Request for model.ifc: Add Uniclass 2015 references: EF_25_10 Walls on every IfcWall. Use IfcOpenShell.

First a look at what the model holds.

```python
import ifcopenshell

model = ifcopenshell.open("model.ifc")
print(model.schema)
print("classifications:", [c.Name for c in model.by_type("IfcClassification")])
for ifc_class in ("IfcDoor", "IfcRoof", "IfcStair", "IfcWall", "IfcWindow"):
    print(ifc_class, len(model.by_type(ifc_class)))
```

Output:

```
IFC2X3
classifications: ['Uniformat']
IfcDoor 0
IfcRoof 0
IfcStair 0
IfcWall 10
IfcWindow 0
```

```python
import ifcopenshell
import ifcopenshell.api.classification

model = ifcopenshell.open("model.ifc")

# IFC2X3 requires Source and Edition and has no link from the project to the system.
system = model.create_entity("IfcClassification", Source="NBS", Edition="2015", Name="Uniclass 2015")

codes = {
    "IfcWall": ("EF_25_10", "Walls"),
}
for ifc_class, (code, name) in codes.items():
    products = model.by_type(ifc_class)
    ifcopenshell.api.classification.add_reference(
        model, products=products, classification=system, identification=code, name=name
    )
    print(code, len(products))

model.write("model_v2.ifc")
```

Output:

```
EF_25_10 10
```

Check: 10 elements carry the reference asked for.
